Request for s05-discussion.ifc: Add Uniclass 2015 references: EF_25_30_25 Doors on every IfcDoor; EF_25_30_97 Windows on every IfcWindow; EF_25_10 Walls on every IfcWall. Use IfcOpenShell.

First a look at what the model holds.

```python
import ifcopenshell

model = ifcopenshell.open("s05-discussion.ifc")
print(model.schema)
print("classifications:", [c.Name for c in model.by_type("IfcClassification")])
for ifc_class in ("IfcDoor", "IfcRoof", "IfcStair", "IfcWall", "IfcWindow"):
    print(ifc_class, len(model.by_type(ifc_class)))
```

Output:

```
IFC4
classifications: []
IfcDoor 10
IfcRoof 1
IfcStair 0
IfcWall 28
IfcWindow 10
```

```python
import ifcopenshell
import ifcopenshell.api.classification

model = ifcopenshell.open("s05-discussion.ifc")

system = ifcopenshell.api.classification.add_classification(model, classification="Uniclass 2015")

codes = {
    "IfcDoor": ("EF_25_30_25", "Doors"),
    "IfcWindow": ("EF_25_30_97", "Windows"),
    "IfcWall": ("EF_25_10", "Walls"),
}
for ifc_class, (code, name) in codes.items():
    products = model.by_type(ifc_class)
    ifcopenshell.api.classification.add_reference(
        model, products=products, classification=system, identification=code, name=name
    )
    print(code, len(products))

model.write("s05-discussion_edited.ifc")
```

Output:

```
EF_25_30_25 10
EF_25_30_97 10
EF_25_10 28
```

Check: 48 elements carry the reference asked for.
